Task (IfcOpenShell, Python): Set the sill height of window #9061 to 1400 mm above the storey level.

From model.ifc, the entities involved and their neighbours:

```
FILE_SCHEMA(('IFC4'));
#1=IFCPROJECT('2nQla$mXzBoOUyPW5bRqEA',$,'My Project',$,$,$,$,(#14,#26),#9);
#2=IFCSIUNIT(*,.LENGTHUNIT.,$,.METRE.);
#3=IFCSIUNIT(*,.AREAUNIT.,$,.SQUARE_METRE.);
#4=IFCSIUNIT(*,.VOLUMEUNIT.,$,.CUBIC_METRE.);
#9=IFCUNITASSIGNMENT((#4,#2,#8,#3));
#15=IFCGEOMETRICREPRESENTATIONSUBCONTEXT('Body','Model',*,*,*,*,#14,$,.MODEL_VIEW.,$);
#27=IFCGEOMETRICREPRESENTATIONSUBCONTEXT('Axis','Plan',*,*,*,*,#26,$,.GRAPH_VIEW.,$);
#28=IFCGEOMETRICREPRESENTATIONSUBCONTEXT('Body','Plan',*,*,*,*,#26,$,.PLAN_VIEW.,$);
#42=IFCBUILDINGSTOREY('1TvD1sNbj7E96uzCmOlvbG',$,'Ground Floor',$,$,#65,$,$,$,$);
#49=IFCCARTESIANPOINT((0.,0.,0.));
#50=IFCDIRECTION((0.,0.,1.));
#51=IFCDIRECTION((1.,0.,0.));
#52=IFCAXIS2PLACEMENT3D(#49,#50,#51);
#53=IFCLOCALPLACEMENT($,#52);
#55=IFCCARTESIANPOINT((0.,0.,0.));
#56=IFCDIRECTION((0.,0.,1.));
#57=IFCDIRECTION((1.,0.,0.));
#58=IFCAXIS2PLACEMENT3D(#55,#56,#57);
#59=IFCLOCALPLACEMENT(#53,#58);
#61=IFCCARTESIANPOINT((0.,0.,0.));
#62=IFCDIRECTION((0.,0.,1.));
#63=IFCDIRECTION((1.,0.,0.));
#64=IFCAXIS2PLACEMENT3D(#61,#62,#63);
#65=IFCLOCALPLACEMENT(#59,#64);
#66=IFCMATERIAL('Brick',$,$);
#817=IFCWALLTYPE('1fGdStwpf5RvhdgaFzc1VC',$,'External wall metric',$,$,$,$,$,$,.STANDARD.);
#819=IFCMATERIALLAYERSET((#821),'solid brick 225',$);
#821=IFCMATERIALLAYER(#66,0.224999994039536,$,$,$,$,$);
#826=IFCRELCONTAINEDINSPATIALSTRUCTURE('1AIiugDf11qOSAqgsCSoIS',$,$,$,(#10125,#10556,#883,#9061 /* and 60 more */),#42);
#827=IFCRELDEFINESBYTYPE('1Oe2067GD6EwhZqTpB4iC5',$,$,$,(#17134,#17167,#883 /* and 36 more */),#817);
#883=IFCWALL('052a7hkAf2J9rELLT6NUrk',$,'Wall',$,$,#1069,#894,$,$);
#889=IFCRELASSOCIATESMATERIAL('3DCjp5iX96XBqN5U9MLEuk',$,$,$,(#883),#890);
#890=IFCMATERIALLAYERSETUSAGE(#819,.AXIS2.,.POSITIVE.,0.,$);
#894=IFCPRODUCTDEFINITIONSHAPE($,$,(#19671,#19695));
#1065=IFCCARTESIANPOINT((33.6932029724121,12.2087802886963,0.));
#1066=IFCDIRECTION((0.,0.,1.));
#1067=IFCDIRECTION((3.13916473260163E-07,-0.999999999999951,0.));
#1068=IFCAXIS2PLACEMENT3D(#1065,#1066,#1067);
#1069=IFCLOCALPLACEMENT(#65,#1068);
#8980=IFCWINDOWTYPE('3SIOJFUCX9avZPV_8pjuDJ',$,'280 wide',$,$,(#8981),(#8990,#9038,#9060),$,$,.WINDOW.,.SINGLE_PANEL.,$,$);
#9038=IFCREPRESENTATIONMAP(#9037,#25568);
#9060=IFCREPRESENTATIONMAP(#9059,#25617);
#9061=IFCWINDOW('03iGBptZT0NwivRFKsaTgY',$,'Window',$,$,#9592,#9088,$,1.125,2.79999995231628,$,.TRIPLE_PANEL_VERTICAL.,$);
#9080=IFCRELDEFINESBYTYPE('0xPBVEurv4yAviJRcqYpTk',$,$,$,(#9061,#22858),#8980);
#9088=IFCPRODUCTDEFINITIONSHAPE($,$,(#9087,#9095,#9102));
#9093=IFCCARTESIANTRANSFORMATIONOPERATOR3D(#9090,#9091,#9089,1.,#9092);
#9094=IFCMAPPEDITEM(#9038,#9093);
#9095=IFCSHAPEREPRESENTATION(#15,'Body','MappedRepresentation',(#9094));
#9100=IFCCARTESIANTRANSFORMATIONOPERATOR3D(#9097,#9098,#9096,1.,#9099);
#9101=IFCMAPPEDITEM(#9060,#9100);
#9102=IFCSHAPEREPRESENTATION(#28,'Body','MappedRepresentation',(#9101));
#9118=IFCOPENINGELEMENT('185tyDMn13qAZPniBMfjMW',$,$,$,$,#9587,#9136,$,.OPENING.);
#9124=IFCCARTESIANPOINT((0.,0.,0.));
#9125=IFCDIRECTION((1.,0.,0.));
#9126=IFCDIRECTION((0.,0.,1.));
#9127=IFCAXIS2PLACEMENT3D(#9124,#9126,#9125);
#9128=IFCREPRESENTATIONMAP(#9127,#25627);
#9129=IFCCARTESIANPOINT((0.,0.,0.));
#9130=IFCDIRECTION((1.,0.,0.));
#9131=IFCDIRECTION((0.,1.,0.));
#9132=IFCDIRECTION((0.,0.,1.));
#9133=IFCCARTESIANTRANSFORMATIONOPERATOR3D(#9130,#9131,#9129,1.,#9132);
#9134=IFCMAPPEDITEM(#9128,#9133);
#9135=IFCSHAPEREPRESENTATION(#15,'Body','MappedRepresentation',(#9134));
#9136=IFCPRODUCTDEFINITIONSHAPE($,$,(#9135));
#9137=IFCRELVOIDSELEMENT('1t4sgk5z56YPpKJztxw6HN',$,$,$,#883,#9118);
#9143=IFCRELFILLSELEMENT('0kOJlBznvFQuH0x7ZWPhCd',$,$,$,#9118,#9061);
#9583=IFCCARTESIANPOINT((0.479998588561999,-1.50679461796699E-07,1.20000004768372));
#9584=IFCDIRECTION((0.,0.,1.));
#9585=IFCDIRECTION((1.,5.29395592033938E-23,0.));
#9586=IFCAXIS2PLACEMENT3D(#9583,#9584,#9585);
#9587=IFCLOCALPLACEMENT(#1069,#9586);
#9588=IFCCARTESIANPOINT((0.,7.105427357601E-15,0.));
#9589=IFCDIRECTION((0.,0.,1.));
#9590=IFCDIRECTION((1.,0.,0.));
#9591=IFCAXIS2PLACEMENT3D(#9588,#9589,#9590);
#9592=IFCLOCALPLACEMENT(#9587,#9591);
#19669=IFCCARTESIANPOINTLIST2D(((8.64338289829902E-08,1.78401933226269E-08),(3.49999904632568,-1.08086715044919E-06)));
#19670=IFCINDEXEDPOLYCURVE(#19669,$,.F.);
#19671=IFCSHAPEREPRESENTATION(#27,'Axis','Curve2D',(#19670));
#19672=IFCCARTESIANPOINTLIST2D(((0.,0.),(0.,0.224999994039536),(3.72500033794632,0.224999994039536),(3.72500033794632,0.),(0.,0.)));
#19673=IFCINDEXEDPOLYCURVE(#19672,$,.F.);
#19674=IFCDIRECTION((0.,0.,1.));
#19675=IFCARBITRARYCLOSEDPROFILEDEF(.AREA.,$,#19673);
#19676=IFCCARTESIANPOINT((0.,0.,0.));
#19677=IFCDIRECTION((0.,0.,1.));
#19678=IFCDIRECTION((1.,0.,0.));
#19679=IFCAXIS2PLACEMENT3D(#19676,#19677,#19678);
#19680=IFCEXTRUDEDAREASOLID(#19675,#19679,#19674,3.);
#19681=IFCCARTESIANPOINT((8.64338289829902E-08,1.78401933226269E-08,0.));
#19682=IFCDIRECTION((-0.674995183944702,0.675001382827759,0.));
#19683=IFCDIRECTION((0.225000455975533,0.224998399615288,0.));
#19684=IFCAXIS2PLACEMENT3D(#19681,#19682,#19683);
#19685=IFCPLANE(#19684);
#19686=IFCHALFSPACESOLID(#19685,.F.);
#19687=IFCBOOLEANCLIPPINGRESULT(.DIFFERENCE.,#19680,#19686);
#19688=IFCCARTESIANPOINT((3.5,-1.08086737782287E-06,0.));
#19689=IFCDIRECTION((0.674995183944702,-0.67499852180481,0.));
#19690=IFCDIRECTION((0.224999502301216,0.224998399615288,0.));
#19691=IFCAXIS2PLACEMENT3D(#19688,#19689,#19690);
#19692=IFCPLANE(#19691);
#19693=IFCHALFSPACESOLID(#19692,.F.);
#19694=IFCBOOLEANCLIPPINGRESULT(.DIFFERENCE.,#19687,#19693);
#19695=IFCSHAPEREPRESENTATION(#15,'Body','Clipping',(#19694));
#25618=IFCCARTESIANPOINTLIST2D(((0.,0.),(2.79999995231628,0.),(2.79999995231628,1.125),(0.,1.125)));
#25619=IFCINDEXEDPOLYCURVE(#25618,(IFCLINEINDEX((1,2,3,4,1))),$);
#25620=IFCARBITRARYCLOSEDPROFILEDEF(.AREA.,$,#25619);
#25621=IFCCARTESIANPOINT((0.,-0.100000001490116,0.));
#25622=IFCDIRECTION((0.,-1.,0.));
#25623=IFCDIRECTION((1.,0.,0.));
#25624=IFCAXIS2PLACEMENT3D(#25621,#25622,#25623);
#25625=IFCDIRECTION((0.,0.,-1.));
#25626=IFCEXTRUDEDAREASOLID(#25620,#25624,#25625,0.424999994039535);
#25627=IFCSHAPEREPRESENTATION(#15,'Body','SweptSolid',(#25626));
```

```python
import numpy as np
import ifcopenshell
import ifcopenshell.api.geometry
import ifcopenshell.geom
import ifcopenshell.util.element
import ifcopenshell.util.placement
import ifcopenshell.util.shape
import ifcopenshell.util.unit

model = ifcopenshell.open("model.ifc")
unit_scale = ifcopenshell.util.unit.calculate_unit_scale(model)

window = model.by_id(9061)
opening = window.FillsVoids[0].RelatingOpeningElement
storey = ifcopenshell.util.element.get_container(window, ifc_class="IfcBuildingStorey")
level = ifcopenshell.util.placement.get_local_placement(storey.ObjectPlacement)[2, 3]

# The opening's origin need not be at the sill, so measure its lowest point.
shape = ifcopenshell.geom.create_shape(ifcopenshell.geom.settings(), opening)
bottom = ifcopenshell.util.shape.get_shape_bottom_elevation(shape, shape.geometry) / unit_scale
dz = level + 1.4 / unit_scale - bottom

shift = np.array([0.0, 0.0, dz])
# The window is placed relative to its opening, so it follows when the opening moves.
matrix = ifcopenshell.util.placement.get_local_placement(opening.ObjectPlacement)
matrix[:3, 3] += shift
ifcopenshell.api.geometry.edit_object_placement(
    model, product=opening, matrix=matrix, is_si=False, should_transform_children=True
)

print(f"moved by {dz * unit_scale:+.3f} m")

model.write("model_edited.ifc")
```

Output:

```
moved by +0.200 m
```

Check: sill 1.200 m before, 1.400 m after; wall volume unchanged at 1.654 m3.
